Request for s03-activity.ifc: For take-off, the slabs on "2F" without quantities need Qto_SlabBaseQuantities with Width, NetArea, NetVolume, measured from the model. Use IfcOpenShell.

First a look at what the model holds.

```python
import ifcopenshell
import ifcopenshell.util.element
import ifcopenshell.util.unit

model = ifcopenshell.open("s03-activity.ifc")
print(model.schema)
for unit_type in ("LENGTHUNIT", "AREAUNIT", "VOLUMEUNIT"):
    print(unit_type, ifcopenshell.util.unit.calculate_unit_scale(model, unit_type))
storey = next(s for s in model.by_type("IfcBuildingStorey") if s.Name == "2F")
slabs = [e for e in ifcopenshell.util.element.get_decomposition(storey) if e.is_a("IfcSlab")]
for e in sorted(slabs, key=lambda e: e.id()):
    print(e.id(), e.is_a(), e.Name, list(ifcopenshell.util.element.get_psets(e, qtos_only=True)), sep=" | ")
```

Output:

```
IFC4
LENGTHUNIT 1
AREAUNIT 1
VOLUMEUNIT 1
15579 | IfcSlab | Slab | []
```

```python
import ifcopenshell
import ifcopenshell.api.pset
import ifcopenshell.geom
import ifcopenshell.util.element
import ifcopenshell.util.shape
import ifcopenshell.util.unit

model = ifcopenshell.open("s03-activity.ifc")
unit_scale = ifcopenshell.util.unit.calculate_unit_scale(model)
area_scale = ifcopenshell.util.unit.calculate_unit_scale(model, "AREAUNIT")
volume_scale = ifcopenshell.util.unit.calculate_unit_scale(model, "VOLUMEUNIT")
settings = ifcopenshell.geom.settings()

storey = next(s for s in model.by_type("IfcBuildingStorey") if s.Name == "2F")
slabs = [e for e in ifcopenshell.util.element.get_decomposition(storey) if e.is_a("IfcSlab")]

for e in sorted(slabs, key=lambda e: e.id()):
    if ifcopenshell.util.element.get_psets(e, qtos_only=True, should_inherit=False):
        continue
    # Geometry comes back in metres, in the element's own axes.
    shape = ifcopenshell.geom.create_shape(settings, e)
    values = {
        "Width": ifcopenshell.util.shape.get_z(shape.geometry) / unit_scale,
        "NetArea": ifcopenshell.util.shape.get_footprint_area(shape.geometry) / area_scale,
        "NetVolume": ifcopenshell.util.shape.get_volume(shape.geometry) / volume_scale,
    }
    qto = ifcopenshell.api.pset.add_qto(model, product=e, name="Qto_SlabBaseQuantities")
    ifcopenshell.api.pset.edit_qto(model, qto=qto, properties=values)
    print(e.id(), {k: round(v, 3) for k, v in values.items()})

model.write("s03-activity_updated.ifc")
```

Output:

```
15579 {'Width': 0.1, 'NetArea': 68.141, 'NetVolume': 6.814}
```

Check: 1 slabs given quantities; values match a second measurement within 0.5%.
